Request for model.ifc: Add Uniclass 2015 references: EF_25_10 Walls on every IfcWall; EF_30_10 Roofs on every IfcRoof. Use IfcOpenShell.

First a look at what the model holds.

```python
import ifcopenshell

model = ifcopenshell.open("model.ifc")
print(model.schema)
print("classifications:", [c.Name for c in model.by_type("IfcClassification")])
for ifc_class in ("IfcDoor", "IfcRoof", "IfcStair", "IfcWall", "IfcWindow"):
    print(ifc_class, len(model.by_type(ifc_class)))
```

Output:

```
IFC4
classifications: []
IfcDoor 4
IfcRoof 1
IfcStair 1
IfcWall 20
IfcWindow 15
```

```python
import ifcopenshell
import ifcopenshell.api.classification

model = ifcopenshell.open("model.ifc")

system = ifcopenshell.api.classification.add_classification(model, classification="Uniclass 2015")

codes = {
    "IfcWall": ("EF_25_10", "Walls"),
    "IfcRoof": ("EF_30_10", "Roofs"),
}
for ifc_class, (code, name) in codes.items():
    products = model.by_type(ifc_class)
    ifcopenshell.api.classification.add_reference(
        model, products=products, classification=system, identification=code, name=name
    )
    print(code, len(products))

model.write("model-out.ifc")
```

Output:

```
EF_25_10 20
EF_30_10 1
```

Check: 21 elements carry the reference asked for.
